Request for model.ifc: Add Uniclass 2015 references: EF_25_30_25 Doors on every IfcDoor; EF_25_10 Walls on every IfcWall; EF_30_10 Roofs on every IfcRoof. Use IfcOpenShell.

First a look at what the model holds.

```python
import ifcopenshell

model = ifcopenshell.open("model.ifc")
print(model.schema)
print("classifications:", [c.Name for c in model.by_type("IfcClassification")])
for ifc_class in ("IfcDoor", "IfcRoof", "IfcStair", "IfcWall", "IfcWindow"):
    print(ifc_class, len(model.by_type(ifc_class)))
```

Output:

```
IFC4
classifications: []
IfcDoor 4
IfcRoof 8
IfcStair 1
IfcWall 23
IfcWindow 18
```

```python
import ifcopenshell
import ifcopenshell.api.classification

model = ifcopenshell.open("model.ifc")

system = ifcopenshell.api.classification.add_classification(model, classification="Uniclass 2015")

codes = {
    "IfcDoor": ("EF_25_30_25", "Doors"),
    "IfcWall": ("EF_25_10", "Walls"),
    "IfcRoof": ("EF_30_10", "Roofs"),
}
for ifc_class, (code, name) in codes.items():
    products = model.by_type(ifc_class)
    ifcopenshell.api.classification.add_reference(
        model, products=products, classification=system, identification=code, name=name
    )
    print(code, len(products))

model.write("model-out.ifc")
```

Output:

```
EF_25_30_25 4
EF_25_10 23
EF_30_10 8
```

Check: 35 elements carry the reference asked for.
